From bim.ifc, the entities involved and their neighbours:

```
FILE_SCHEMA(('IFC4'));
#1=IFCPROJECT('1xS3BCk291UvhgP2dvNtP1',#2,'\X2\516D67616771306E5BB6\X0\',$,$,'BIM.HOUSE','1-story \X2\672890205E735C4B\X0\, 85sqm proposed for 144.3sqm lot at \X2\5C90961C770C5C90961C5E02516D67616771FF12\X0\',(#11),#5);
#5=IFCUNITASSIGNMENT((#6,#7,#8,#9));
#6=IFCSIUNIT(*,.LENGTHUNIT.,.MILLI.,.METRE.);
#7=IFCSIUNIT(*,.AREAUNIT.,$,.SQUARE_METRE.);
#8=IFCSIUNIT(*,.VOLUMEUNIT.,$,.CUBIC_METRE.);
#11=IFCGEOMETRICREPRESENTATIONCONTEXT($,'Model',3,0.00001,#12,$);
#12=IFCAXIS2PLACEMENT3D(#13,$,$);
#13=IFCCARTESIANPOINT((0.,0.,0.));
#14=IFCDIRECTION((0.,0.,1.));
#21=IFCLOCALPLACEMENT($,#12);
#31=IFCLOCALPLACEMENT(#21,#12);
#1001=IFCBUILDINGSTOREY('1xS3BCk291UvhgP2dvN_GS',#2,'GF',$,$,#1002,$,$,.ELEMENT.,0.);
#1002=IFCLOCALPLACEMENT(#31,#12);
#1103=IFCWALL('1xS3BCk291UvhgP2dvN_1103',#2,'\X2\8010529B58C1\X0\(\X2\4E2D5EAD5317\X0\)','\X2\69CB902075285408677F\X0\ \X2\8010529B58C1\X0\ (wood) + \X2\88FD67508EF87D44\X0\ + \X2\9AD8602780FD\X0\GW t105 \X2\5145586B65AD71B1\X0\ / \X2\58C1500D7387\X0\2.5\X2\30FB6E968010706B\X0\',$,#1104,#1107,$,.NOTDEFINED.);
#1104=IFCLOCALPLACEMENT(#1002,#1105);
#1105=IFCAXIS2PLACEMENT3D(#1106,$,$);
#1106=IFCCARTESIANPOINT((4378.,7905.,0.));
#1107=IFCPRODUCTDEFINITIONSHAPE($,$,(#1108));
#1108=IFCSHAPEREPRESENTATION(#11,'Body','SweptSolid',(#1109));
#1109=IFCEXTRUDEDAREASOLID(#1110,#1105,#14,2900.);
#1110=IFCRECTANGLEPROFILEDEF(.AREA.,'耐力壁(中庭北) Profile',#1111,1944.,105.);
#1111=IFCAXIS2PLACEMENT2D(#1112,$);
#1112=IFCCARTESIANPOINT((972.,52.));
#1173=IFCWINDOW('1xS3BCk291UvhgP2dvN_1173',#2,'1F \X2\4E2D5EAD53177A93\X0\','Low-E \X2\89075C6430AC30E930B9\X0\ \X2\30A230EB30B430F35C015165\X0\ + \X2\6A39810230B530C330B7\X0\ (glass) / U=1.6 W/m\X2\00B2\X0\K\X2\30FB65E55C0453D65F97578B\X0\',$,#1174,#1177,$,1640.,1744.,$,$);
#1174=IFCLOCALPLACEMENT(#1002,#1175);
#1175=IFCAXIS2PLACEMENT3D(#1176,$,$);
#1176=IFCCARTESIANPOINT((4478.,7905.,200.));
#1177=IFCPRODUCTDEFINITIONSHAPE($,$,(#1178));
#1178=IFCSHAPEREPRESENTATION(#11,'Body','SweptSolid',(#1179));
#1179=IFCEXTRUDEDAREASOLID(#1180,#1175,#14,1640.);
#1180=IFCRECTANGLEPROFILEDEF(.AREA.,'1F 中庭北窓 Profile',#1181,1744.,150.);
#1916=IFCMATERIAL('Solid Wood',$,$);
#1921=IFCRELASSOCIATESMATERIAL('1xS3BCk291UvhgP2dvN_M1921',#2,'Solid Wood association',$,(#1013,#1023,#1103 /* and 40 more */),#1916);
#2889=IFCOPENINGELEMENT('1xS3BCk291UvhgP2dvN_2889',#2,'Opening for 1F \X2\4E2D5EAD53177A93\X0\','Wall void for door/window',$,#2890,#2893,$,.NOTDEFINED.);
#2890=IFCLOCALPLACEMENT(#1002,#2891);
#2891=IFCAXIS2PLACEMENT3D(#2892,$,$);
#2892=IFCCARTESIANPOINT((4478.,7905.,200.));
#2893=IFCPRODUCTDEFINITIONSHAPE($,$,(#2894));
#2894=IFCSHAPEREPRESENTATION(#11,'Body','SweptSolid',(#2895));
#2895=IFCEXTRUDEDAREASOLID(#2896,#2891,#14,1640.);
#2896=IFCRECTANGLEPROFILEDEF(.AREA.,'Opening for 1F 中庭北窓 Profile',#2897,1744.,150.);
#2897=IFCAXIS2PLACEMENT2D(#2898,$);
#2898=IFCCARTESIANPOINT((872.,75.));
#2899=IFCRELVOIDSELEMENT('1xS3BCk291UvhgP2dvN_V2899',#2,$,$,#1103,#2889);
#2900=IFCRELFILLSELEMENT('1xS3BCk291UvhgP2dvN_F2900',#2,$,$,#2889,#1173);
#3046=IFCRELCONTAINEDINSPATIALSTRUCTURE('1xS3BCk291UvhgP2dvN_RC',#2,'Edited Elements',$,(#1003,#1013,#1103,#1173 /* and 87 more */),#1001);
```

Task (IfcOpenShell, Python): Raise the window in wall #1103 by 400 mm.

```python
import numpy as np
import ifcopenshell
import ifcopenshell.api.geometry
import ifcopenshell.util.placement
import ifcopenshell.util.unit

model = ifcopenshell.open("bim.ifc")
unit_scale = ifcopenshell.util.unit.calculate_unit_scale(model)

window = model.by_guid("1xS3BCk291UvhgP2dvN_1173")
opening = window.FillsVoids[0].RelatingOpeningElement
dz = 0.4 / unit_scale

shift = np.array([0.0, 0.0, dz])
# The window is not placed relative to its opening, so move both.
for product in (opening, window):
    matrix = ifcopenshell.util.placement.get_local_placement(product.ObjectPlacement)
    matrix[:3, 3] += shift
    ifcopenshell.api.geometry.edit_object_placement(model, product=product, matrix=matrix, is_si=False)

print(f"moved by {dz * unit_scale:+.3f} m")

model.write("bim_updated.ifc")
```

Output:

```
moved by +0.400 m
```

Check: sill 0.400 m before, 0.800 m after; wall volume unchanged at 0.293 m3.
